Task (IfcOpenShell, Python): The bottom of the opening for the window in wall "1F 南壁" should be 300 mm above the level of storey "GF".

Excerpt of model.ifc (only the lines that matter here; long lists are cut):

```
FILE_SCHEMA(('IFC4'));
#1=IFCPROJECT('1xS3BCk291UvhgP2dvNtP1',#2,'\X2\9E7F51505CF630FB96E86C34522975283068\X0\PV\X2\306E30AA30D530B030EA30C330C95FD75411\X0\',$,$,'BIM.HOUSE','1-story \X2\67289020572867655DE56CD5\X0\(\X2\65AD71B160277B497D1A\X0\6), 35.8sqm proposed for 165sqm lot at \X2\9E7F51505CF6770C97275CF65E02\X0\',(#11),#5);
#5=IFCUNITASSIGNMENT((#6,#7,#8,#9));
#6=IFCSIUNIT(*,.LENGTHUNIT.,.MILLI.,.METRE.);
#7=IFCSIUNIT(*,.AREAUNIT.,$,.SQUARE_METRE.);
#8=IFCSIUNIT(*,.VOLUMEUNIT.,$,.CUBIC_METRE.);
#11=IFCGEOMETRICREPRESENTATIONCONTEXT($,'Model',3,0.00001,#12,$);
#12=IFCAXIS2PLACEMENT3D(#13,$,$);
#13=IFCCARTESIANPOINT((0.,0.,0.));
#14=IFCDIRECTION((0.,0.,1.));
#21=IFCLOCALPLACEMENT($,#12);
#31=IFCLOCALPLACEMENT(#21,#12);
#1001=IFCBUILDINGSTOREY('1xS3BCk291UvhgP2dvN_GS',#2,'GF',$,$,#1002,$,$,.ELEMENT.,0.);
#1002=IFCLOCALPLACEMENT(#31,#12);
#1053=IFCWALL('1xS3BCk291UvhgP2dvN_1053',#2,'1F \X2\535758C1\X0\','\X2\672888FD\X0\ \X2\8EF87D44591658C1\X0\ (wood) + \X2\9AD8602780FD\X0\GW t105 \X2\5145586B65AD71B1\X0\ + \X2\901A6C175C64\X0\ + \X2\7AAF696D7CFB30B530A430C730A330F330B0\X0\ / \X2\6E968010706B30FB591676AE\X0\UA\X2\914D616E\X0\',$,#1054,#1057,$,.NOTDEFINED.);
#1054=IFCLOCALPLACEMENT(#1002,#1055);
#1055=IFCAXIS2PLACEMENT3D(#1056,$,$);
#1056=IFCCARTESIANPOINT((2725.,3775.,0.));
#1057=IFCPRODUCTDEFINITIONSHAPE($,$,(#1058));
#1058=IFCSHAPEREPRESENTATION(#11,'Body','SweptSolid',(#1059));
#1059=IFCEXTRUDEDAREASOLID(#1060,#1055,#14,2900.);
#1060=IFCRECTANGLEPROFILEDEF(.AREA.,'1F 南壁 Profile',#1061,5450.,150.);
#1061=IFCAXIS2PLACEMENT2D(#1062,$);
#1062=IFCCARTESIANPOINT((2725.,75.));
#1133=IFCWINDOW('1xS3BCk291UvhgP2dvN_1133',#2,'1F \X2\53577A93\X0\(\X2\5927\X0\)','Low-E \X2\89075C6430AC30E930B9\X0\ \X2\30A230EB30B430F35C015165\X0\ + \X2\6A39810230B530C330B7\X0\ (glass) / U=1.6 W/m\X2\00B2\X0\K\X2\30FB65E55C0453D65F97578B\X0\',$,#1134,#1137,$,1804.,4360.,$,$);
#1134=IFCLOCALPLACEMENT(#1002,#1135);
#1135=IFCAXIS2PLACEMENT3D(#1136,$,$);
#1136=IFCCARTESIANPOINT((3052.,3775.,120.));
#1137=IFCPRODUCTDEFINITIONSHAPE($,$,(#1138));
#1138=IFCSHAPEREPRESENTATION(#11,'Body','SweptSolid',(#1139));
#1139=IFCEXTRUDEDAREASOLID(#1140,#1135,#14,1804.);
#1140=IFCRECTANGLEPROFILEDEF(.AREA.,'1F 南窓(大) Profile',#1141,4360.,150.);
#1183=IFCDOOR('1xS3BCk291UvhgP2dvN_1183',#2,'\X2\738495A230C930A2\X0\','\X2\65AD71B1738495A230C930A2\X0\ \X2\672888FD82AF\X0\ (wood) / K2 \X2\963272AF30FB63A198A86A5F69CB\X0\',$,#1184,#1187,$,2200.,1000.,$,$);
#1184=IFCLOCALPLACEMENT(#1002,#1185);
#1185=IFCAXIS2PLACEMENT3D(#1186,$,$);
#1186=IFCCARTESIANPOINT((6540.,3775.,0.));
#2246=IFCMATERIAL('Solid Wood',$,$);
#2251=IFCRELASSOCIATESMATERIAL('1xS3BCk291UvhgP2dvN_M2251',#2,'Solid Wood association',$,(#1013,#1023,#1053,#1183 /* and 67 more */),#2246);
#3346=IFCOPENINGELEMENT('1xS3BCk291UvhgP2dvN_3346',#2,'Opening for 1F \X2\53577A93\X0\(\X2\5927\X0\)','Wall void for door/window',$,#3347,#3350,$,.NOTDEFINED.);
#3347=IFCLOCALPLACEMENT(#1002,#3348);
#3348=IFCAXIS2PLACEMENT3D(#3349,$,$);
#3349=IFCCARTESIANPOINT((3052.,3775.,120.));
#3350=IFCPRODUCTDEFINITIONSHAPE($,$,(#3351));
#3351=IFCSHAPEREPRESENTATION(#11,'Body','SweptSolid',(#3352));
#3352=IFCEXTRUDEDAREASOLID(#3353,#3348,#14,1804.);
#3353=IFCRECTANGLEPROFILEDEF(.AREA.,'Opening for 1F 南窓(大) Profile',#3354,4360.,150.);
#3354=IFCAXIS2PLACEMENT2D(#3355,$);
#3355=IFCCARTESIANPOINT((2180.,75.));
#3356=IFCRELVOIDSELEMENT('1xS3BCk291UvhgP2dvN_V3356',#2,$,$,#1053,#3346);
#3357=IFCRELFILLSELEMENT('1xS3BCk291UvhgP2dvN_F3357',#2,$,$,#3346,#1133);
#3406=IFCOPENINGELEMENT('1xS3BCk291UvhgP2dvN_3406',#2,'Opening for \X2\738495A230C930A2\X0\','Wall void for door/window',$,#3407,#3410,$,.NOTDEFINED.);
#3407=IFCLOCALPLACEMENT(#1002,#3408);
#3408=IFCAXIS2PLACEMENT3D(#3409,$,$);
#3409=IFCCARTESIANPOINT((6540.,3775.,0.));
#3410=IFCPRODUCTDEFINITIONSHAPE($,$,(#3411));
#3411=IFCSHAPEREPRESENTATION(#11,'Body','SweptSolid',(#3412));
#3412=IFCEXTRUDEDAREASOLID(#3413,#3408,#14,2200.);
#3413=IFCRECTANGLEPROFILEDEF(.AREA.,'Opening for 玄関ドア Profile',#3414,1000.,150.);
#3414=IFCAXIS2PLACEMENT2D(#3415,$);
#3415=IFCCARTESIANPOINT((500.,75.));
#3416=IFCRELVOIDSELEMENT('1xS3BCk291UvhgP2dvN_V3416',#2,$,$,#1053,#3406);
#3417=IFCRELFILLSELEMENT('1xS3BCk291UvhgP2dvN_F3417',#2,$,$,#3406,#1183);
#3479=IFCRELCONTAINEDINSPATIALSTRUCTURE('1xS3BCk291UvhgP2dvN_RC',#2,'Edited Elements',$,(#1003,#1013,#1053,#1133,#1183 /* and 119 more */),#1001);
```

```python
import numpy as np
import ifcopenshell
import ifcopenshell.api.geometry
import ifcopenshell.geom
import ifcopenshell.util.element
import ifcopenshell.util.placement
import ifcopenshell.util.shape
import ifcopenshell.util.unit

model = ifcopenshell.open("model.ifc")
unit_scale = ifcopenshell.util.unit.calculate_unit_scale(model)

window = model.by_guid("1xS3BCk291UvhgP2dvN_1133")
opening = window.FillsVoids[0].RelatingOpeningElement
storey = ifcopenshell.util.element.get_container(window, ifc_class="IfcBuildingStorey")
level = ifcopenshell.util.placement.get_local_placement(storey.ObjectPlacement)[2, 3]

# The opening's origin need not be at the sill, so measure its lowest point.
shape = ifcopenshell.geom.create_shape(ifcopenshell.geom.settings(), opening)
bottom = ifcopenshell.util.shape.get_shape_bottom_elevation(shape, shape.geometry) / unit_scale
dz = level + 0.3 / unit_scale - bottom

shift = np.array([0.0, 0.0, dz])
# The window is not placed relative to its opening, so move both.
for product in (opening, window):
    matrix = ifcopenshell.util.placement.get_local_placement(product.ObjectPlacement)
    matrix[:3, 3] += shift
    ifcopenshell.api.geometry.edit_object_placement(model, product=product, matrix=matrix, is_si=False)

print(f"moved by {dz * unit_scale:+.3f} m")

model.write("model_updated.ifc")
```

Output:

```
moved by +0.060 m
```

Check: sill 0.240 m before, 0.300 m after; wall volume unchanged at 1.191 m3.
